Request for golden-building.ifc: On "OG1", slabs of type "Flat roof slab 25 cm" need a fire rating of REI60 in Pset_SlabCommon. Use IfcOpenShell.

First a look at what the model holds.

```python
import ifcopenshell
import ifcopenshell.util.element

model = ifcopenshell.open("golden-building.ifc")
print(model.schema)
storey = next(s for s in model.by_type("IfcBuildingStorey") if s.Name == "OG1")
slabs = [e for e in ifcopenshell.util.element.get_decomposition(storey) if e.is_a("IfcSlab")]
seen = {}
for e in slabs:
    element_type = ifcopenshell.util.element.get_type(e)
    key = (element_type.Name if element_type != e and element_type else None, ifcopenshell.util.element.get_pset(e, "Pset_SlabCommon", "FireRating"))
    seen[key] = seen.get(key, 0) + 1
for (name, value), count in sorted(seen.items(), key=str):
    print(count, "x", name, "|", value)
```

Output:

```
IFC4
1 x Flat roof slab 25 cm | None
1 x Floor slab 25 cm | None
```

```python
import ifcopenshell
import ifcopenshell.api.pset
import ifcopenshell.util.element

model = ifcopenshell.open("golden-building.ifc")

storey = next(s for s in model.by_type("IfcBuildingStorey") if s.Name == "OG1")
slabs = [e for e in ifcopenshell.util.element.get_decomposition(storey) if e.is_a("IfcSlab")]

count = 0
for e in slabs:
    element_type = ifcopenshell.util.element.get_type(e)
    if element_type in (None, e) or element_type.Name != "Flat roof slab 25 cm":
        continue
    # add_pset returns the element's existing set when there is one.
    pset = ifcopenshell.api.pset.add_pset(model, product=e, name="Pset_SlabCommon")
    ifcopenshell.api.pset.edit_pset(model, pset=pset, properties={"FireRating": "REI60"})
    count += 1

print(count, "slabs updated")

model.write("golden-building-out.ifc")
```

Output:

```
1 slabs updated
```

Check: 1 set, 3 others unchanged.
